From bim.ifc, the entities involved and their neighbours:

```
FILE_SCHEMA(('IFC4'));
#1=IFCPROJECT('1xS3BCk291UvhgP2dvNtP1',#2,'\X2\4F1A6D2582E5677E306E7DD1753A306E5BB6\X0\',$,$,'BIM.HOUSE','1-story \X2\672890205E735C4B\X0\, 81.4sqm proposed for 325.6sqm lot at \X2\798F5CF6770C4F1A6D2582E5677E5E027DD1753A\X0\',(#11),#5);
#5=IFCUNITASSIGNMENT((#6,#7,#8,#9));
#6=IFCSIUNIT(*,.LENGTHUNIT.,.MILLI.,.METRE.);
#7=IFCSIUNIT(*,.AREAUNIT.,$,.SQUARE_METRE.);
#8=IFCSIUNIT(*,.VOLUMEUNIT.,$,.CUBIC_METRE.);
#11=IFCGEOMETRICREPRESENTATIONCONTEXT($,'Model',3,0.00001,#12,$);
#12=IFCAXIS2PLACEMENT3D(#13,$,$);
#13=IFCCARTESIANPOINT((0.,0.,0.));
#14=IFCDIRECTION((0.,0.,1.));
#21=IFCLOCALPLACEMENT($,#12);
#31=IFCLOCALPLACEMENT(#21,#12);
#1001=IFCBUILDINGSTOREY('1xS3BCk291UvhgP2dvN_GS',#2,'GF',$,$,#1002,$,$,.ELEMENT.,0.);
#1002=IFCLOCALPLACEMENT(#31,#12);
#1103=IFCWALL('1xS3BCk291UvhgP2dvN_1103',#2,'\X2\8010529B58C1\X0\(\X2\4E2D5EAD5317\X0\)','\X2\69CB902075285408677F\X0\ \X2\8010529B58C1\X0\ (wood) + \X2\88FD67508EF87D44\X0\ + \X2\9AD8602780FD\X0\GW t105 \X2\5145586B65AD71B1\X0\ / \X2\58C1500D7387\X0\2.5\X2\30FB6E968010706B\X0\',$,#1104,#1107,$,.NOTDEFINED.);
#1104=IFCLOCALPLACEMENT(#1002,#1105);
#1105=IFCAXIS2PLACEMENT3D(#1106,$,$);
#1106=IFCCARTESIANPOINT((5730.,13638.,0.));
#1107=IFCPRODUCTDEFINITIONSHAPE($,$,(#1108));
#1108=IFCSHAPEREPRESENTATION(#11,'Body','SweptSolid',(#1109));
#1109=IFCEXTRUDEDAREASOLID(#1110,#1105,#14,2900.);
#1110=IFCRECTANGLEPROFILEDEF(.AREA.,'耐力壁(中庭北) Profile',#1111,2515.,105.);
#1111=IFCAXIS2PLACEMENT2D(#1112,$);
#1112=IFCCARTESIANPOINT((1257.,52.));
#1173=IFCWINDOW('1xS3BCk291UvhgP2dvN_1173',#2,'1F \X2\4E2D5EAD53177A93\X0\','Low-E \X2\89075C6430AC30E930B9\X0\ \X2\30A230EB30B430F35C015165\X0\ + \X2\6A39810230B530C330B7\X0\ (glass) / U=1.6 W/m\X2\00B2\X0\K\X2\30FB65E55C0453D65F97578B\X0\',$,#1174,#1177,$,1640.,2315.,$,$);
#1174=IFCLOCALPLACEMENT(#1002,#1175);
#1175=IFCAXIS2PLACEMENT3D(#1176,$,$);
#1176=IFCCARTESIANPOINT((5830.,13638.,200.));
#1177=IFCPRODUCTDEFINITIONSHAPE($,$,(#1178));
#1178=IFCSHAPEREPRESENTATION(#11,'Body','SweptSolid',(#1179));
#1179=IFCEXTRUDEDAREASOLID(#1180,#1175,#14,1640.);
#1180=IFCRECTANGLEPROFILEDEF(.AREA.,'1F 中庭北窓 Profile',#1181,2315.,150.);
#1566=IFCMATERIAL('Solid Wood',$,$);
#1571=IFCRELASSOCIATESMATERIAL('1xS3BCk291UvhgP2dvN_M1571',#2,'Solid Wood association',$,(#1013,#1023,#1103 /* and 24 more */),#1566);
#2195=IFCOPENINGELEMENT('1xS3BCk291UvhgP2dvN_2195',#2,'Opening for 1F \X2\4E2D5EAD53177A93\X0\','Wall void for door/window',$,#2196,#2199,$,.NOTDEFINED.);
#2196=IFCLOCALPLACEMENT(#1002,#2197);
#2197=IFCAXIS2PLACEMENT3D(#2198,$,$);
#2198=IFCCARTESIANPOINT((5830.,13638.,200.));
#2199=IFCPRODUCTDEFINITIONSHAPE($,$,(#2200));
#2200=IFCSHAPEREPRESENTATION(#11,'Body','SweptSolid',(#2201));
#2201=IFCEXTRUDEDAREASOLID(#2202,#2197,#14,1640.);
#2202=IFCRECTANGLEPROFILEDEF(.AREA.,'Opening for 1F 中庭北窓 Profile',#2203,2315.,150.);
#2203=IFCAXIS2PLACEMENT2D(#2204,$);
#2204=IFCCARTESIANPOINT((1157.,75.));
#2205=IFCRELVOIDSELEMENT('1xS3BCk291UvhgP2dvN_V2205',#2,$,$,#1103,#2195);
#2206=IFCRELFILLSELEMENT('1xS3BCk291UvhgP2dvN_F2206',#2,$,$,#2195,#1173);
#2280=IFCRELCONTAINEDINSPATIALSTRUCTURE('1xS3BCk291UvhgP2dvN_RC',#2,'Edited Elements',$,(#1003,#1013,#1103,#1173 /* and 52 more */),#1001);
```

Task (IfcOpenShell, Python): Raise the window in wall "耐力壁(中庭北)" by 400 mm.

```python
import numpy as np
import ifcopenshell
import ifcopenshell.api.geometry
import ifcopenshell.util.placement
import ifcopenshell.util.unit

model = ifcopenshell.open("bim.ifc")
unit_scale = ifcopenshell.util.unit.calculate_unit_scale(model)

window = model.by_guid("1xS3BCk291UvhgP2dvN_1173")
opening = window.FillsVoids[0].RelatingOpeningElement
dz = 400.0

shift = np.array([0.0, 0.0, dz])
# The window is not placed relative to its opening, so move both.
for product in (opening, window):
    matrix = ifcopenshell.util.placement.get_local_placement(product.ObjectPlacement)
    matrix[:3, 3] += shift
    ifcopenshell.api.geometry.edit_object_placement(model, product=product, matrix=matrix, is_si=False)

print(f"moved by {dz * unit_scale:+.3f} m")

model.write("bim-out.ifc")
```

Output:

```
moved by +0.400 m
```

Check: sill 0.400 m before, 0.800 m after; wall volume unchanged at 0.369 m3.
